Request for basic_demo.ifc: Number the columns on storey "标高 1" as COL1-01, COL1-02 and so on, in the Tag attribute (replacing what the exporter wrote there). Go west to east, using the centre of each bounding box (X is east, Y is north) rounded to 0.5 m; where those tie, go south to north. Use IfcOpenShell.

First a look at what the model holds.

```python
import ifcopenshell
import ifcopenshell.util.element
import ifcopenshell.util.placement

model = ifcopenshell.open("basic_demo.ifc")
print(model.schema)
storey = next(s for s in model.by_type("IfcBuildingStorey") if s.Name == "标高 1")
columns = [e for e in ifcopenshell.util.element.get_decomposition(storey) if e.is_a("IfcColumn")]
for e in sorted(columns, key=lambda e: e.id()):
    origin = ifcopenshell.util.placement.get_local_placement(e.ObjectPlacement)[:3, 3]
    print(e.id(), e.Tag, e.Name, origin.round(2) + 0.0, sep=" | ")
```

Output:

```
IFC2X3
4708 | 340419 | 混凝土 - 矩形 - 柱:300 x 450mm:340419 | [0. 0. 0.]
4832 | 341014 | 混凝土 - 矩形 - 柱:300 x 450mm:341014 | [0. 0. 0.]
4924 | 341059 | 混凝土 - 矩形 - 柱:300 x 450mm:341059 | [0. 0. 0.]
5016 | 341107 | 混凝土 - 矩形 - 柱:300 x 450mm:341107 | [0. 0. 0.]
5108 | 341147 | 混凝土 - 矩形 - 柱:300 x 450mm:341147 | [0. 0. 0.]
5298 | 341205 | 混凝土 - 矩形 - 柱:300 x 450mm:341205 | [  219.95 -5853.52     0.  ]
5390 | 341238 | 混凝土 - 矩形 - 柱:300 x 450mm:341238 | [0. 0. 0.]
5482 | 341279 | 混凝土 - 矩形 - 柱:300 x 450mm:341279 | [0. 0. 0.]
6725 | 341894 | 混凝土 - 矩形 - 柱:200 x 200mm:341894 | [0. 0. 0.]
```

```python
import ifcopenshell
import ifcopenshell.geom
import ifcopenshell.util.element
import ifcopenshell.util.shape

model = ifcopenshell.open("basic_demo.ifc")
settings = ifcopenshell.geom.settings()
settings.set("use-world-coords", True)


def centre(element):
    shape = ifcopenshell.geom.create_shape(settings, element)
    return ifcopenshell.util.shape.get_bbox_centroid(shape.geometry)


storey = next(s for s in model.by_type("IfcBuildingStorey") if s.Name == "标高 1")
columns = [e for e in ifcopenshell.util.element.get_decomposition(storey) if e.is_a("IfcColumn")]

# Insertion points can sit at a corner or the storey origin, so sort by the geometry (in metres).
centres = {e: centre(e) for e in columns}
columns.sort(key=lambda e: (round(centres[e][0] / 0.5), centres[e][1]))

for i, e in enumerate(columns, start=1):
    number = f"COL1-{i:02d}"
    e.Tag = number
    print(e.id(), number)

model.write("basic_demo_edited.ifc")
```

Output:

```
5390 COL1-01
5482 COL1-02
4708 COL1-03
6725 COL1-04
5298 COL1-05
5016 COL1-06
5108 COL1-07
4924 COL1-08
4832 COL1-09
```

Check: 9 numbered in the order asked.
